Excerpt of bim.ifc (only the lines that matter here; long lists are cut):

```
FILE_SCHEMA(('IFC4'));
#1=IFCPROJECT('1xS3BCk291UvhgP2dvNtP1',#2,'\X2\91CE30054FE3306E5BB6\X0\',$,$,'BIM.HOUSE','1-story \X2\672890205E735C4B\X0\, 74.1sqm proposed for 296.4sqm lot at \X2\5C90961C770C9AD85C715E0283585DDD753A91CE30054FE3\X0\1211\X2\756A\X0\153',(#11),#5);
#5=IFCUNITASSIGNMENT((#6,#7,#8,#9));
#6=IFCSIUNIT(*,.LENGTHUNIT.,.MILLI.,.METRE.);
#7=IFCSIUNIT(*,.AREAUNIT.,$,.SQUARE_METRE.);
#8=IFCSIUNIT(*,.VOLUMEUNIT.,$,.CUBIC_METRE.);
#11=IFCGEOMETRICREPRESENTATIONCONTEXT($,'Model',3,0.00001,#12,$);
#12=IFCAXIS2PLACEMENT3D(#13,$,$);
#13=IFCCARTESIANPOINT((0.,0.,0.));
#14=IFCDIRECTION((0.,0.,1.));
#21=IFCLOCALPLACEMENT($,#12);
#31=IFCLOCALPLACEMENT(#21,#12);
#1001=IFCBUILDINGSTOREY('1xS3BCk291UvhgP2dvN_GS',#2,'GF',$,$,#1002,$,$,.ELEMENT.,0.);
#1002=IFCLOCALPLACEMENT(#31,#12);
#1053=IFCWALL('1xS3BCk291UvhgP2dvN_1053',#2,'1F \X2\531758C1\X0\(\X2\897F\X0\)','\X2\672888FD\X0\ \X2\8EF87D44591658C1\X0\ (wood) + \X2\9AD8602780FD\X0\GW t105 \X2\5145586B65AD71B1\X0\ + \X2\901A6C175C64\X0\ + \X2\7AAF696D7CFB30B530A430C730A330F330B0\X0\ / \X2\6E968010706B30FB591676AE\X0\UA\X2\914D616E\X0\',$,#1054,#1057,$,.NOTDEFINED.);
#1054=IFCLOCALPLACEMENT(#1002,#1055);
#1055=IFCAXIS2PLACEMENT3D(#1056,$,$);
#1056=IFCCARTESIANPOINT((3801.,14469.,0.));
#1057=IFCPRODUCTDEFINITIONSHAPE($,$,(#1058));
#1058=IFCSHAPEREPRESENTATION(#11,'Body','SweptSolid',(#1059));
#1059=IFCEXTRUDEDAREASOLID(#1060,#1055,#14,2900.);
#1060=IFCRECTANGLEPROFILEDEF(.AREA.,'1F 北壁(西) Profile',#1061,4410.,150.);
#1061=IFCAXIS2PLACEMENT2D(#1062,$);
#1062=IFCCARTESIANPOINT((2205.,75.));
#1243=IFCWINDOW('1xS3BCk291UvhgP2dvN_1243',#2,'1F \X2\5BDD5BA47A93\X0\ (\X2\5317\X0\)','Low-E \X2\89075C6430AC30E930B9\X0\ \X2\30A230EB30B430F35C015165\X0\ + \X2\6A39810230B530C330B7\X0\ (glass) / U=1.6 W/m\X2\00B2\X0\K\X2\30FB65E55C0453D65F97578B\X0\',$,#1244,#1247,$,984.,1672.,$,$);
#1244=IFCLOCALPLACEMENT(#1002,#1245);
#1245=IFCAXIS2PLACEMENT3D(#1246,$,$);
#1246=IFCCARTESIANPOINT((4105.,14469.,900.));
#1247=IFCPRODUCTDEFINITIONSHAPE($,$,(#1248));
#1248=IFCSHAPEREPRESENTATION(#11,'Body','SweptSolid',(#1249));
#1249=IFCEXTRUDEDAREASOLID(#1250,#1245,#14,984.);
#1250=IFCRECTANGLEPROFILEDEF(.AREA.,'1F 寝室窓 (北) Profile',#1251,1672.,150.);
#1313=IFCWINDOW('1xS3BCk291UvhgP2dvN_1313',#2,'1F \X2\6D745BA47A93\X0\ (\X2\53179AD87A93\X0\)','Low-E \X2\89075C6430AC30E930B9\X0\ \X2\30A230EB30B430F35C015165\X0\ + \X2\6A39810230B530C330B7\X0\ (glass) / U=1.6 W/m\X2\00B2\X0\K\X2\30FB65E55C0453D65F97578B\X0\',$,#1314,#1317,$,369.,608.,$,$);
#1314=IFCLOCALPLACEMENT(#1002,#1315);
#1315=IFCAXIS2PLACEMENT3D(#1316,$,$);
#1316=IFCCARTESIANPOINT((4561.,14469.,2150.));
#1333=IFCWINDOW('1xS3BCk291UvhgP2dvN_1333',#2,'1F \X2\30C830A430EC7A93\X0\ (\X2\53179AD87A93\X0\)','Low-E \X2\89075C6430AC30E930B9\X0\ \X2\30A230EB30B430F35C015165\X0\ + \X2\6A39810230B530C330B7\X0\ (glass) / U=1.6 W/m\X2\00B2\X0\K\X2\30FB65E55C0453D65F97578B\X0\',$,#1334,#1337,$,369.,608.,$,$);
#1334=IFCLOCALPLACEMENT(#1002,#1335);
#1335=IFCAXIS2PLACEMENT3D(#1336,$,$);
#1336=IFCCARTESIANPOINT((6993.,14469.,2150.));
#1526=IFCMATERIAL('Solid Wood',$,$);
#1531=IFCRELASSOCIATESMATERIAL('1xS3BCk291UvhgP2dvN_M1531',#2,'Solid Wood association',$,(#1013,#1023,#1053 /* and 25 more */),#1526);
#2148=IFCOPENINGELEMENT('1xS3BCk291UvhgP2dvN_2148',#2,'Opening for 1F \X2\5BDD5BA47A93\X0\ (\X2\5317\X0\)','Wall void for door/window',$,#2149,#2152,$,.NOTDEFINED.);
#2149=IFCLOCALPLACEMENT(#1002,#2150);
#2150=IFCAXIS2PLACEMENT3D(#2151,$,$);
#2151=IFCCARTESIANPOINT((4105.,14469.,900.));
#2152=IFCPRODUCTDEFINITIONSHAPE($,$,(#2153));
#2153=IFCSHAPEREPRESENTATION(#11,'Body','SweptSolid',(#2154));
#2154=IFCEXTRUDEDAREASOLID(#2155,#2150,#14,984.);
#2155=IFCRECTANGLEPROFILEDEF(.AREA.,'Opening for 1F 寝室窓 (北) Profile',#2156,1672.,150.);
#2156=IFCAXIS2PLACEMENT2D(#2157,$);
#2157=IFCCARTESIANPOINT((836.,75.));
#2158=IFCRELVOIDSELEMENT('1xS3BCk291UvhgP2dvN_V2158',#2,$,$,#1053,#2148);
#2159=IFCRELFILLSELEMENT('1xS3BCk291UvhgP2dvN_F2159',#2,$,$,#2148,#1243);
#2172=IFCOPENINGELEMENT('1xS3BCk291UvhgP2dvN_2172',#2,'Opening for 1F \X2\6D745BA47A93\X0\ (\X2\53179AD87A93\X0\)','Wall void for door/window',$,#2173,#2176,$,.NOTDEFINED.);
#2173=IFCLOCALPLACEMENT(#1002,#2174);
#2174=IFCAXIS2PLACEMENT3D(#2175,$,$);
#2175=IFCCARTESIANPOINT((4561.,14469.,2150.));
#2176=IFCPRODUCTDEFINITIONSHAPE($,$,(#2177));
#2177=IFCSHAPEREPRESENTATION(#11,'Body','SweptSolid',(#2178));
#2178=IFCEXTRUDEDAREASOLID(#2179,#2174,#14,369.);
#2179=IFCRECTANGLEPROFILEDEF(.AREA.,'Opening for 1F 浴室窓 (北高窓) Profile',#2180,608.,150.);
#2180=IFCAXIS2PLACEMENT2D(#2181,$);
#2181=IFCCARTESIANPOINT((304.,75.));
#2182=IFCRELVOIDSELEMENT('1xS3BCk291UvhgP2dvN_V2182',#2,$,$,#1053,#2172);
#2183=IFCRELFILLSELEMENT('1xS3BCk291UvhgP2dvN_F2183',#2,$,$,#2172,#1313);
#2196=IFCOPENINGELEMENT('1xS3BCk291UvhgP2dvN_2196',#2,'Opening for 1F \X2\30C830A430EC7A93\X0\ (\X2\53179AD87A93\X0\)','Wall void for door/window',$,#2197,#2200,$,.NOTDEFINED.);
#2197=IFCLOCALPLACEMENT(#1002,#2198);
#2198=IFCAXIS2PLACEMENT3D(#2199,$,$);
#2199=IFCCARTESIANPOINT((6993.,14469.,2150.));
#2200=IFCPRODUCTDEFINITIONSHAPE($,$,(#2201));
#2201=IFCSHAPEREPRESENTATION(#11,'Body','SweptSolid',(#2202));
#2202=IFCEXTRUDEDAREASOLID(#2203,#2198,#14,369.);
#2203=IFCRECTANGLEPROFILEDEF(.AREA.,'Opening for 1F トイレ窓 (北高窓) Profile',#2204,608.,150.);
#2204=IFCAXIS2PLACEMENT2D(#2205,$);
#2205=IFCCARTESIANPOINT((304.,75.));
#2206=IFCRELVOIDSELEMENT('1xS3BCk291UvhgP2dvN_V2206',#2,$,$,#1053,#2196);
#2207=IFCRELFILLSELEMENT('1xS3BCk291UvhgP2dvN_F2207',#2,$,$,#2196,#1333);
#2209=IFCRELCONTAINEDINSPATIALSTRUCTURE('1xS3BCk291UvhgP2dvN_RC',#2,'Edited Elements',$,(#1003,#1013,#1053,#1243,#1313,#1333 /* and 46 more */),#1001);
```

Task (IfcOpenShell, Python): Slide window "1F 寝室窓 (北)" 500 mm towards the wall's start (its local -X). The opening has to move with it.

```python
import ifcopenshell
import ifcopenshell.api.geometry
import ifcopenshell.util.placement
import ifcopenshell.util.unit

model = ifcopenshell.open("bim.ifc")
unit_scale = ifcopenshell.util.unit.calculate_unit_scale(model)

window = model.by_id(1243)
opening = window.FillsVoids[0].RelatingOpeningElement
wall = opening.VoidsElements[0].RelatingBuildingElement

wall_matrix = ifcopenshell.util.placement.get_local_placement(wall.ObjectPlacement)
shift = wall_matrix[:3, 0] * -0.5 / unit_scale
before = ifcopenshell.util.placement.get_local_placement(window.ObjectPlacement)[:3, 3].copy()

# The window is not placed relative to its opening, so move both.
for product in (opening, window):
    matrix = ifcopenshell.util.placement.get_local_placement(product.ObjectPlacement)
    matrix[:3, 3] += shift
    ifcopenshell.api.geometry.edit_object_placement(model, product=product, matrix=matrix, is_si=False)

after = ifcopenshell.util.placement.get_local_placement(window.ObjectPlacement)[:3, 3]
print("window moved by", (after - before).round(3) + 0.0)

model.write("bim_v2.ifc")
```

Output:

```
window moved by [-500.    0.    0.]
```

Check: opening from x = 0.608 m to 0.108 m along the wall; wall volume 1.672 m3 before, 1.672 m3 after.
